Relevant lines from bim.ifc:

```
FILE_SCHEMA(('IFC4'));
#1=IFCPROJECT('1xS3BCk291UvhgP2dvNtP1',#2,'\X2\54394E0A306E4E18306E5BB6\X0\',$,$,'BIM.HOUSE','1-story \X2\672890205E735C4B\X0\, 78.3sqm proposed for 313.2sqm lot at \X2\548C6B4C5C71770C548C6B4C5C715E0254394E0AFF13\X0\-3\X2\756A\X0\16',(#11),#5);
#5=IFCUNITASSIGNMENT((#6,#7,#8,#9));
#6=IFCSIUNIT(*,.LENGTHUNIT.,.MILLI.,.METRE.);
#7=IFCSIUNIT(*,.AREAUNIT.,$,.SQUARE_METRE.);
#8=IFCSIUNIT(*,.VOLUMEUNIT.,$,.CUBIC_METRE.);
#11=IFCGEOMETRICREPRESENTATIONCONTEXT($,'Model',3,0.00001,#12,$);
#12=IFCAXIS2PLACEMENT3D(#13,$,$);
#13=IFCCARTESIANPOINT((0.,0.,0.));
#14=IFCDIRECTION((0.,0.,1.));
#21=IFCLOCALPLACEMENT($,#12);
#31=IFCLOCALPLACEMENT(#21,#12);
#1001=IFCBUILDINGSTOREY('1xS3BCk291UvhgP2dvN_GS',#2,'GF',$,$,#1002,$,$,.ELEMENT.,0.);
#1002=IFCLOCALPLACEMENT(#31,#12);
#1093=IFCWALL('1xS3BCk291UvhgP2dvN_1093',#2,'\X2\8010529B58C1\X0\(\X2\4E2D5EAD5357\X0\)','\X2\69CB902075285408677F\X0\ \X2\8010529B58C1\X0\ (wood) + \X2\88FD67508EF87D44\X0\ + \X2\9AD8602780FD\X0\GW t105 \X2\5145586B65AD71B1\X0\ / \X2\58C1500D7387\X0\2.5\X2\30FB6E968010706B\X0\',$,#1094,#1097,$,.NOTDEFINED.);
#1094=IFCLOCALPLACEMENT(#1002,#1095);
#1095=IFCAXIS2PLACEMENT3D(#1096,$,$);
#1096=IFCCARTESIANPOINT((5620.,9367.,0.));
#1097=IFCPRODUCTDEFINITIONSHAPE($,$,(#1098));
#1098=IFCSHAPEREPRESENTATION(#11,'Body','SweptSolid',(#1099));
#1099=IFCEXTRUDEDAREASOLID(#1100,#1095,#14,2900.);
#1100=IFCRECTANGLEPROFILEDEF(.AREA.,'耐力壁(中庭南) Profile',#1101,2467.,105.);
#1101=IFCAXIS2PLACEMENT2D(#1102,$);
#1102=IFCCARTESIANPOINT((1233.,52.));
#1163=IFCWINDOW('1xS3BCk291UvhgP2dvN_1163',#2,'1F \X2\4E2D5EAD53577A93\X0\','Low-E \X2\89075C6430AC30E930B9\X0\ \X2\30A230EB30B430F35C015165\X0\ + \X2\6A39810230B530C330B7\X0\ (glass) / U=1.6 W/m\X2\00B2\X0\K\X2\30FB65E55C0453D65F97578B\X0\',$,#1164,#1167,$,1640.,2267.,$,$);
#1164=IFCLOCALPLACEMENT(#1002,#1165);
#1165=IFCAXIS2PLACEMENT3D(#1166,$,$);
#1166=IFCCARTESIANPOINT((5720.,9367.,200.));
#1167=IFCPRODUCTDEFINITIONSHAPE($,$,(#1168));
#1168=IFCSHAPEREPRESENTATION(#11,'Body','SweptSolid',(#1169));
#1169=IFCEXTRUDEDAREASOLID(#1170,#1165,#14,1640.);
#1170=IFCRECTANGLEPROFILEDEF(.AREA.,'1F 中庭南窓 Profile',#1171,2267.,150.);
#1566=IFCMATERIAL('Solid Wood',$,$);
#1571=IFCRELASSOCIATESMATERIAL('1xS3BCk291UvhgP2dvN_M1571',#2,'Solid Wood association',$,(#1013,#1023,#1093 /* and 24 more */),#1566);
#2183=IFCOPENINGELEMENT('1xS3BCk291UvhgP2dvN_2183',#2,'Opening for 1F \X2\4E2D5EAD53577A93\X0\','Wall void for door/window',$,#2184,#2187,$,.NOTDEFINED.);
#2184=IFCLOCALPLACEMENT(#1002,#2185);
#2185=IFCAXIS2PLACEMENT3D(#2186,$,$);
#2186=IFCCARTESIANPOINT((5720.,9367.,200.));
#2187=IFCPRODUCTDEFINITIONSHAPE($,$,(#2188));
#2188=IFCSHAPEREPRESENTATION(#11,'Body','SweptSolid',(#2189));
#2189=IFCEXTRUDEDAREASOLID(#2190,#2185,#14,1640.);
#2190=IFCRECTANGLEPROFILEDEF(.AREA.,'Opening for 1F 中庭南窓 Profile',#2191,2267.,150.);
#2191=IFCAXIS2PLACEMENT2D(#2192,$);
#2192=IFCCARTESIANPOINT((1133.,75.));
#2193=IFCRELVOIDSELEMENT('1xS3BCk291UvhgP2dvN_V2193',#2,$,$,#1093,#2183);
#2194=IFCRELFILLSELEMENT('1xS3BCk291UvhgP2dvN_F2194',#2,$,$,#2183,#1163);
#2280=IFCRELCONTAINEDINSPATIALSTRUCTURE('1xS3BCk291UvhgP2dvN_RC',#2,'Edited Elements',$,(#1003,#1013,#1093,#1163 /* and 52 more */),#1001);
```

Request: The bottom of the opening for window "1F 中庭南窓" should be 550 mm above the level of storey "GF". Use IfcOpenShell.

```python
import numpy as np
import ifcopenshell
import ifcopenshell.api.geometry
import ifcopenshell.geom
import ifcopenshell.util.element
import ifcopenshell.util.placement
import ifcopenshell.util.shape
import ifcopenshell.util.unit

model = ifcopenshell.open("bim.ifc")
unit_scale = ifcopenshell.util.unit.calculate_unit_scale(model)

window = model.by_guid("1xS3BCk291UvhgP2dvN_1163")
opening = window.FillsVoids[0].RelatingOpeningElement
storey = ifcopenshell.util.element.get_container(window, ifc_class="IfcBuildingStorey")
level = ifcopenshell.util.placement.get_local_placement(storey.ObjectPlacement)[2, 3]

# The opening's origin need not be at the sill, so measure its lowest point.
shape = ifcopenshell.geom.create_shape(ifcopenshell.geom.settings(), opening)
bottom = ifcopenshell.util.shape.get_shape_bottom_elevation(shape, shape.geometry) / unit_scale
dz = level + 0.55 / unit_scale - bottom

shift = np.array([0.0, 0.0, dz])
# The window is not placed relative to its opening, so move both.
for product in (opening, window):
    matrix = ifcopenshell.util.placement.get_local_placement(product.ObjectPlacement)
    matrix[:3, 3] += shift
    ifcopenshell.api.geometry.edit_object_placement(model, product=product, matrix=matrix, is_si=False)

print(f"moved by {dz * unit_scale:+.3f} m")

model.write("bim_rev.ifc")
```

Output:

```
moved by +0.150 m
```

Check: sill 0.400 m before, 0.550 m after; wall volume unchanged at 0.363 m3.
